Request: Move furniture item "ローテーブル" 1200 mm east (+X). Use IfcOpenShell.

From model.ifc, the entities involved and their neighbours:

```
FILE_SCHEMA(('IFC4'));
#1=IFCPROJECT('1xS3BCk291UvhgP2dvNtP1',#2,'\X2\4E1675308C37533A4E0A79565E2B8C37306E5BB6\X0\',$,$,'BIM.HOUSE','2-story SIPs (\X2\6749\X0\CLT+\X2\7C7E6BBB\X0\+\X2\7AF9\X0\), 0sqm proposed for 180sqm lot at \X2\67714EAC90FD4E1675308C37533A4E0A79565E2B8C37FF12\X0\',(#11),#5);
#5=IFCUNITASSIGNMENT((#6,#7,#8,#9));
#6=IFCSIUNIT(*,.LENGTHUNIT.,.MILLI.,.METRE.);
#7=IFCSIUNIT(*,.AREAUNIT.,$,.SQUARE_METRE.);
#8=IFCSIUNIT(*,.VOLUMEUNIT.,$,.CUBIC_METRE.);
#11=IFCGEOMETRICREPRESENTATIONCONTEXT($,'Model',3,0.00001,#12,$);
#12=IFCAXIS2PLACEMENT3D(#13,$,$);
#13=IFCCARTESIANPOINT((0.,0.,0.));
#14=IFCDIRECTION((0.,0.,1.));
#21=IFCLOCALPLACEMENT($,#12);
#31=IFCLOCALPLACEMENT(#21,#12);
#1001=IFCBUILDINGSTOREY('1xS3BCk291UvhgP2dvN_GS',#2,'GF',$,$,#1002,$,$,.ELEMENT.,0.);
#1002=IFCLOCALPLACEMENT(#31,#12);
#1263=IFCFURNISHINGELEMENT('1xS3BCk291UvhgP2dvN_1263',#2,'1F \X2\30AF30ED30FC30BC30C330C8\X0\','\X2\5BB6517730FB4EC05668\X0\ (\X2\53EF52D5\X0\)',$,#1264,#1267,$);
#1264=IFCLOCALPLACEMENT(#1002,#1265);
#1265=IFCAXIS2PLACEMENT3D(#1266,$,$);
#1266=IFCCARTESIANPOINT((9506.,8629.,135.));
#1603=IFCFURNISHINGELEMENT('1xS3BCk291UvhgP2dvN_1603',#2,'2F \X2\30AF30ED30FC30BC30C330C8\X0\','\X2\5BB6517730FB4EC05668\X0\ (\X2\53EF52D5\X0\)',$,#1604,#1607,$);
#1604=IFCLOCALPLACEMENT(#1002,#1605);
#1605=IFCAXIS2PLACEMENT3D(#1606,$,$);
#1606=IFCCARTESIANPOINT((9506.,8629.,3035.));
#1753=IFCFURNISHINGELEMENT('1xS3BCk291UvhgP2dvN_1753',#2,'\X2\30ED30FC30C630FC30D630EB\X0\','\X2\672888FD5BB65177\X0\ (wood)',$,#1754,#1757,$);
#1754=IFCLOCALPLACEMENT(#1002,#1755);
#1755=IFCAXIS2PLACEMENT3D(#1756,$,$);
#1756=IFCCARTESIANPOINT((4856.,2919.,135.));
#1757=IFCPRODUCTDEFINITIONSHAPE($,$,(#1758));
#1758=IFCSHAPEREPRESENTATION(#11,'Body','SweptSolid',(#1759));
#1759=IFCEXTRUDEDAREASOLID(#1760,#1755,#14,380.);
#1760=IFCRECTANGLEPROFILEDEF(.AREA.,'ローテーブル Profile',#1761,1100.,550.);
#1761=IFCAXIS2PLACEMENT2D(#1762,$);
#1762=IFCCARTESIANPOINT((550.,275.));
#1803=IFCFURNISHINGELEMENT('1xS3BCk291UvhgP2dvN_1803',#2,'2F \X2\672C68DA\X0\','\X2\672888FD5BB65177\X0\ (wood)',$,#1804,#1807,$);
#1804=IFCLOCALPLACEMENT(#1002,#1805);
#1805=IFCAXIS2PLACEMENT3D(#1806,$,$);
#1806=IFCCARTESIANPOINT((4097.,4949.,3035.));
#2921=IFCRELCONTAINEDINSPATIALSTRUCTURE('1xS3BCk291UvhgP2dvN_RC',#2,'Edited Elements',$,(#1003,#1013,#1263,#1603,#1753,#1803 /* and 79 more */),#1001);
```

```python
import ifcopenshell
import ifcopenshell.api.geometry
import ifcopenshell.util.placement
import ifcopenshell.util.unit

model = ifcopenshell.open("model.ifc")
unit_scale = ifcopenshell.util.unit.calculate_unit_scale(model)

item = model.by_id(1753)
matrix = ifcopenshell.util.placement.get_local_placement(item.ObjectPlacement)
matrix[0, 3] += 1.2 / unit_scale
ifcopenshell.api.geometry.edit_object_placement(model, product=item, matrix=matrix, is_si=False)

print(ifcopenshell.util.placement.get_local_placement(item.ObjectPlacement).round(3) + 0.0)

model.write("model_edited.ifc")
```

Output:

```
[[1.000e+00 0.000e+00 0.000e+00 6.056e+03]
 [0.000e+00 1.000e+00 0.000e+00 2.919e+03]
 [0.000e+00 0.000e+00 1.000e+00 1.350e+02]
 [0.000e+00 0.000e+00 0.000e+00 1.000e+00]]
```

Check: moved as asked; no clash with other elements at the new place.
